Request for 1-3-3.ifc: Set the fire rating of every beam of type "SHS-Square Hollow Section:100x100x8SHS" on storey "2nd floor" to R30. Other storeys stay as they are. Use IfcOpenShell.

First a look at what the model holds.

```python
import ifcopenshell
import ifcopenshell.util.element

model = ifcopenshell.open("1-3-3.ifc")
print(model.schema)
storey = next(s for s in model.by_type("IfcBuildingStorey") if s.Name == "2nd floor")
beams = [e for e in ifcopenshell.util.element.get_decomposition(storey) if e.is_a("IfcBeam")]
seen = {}
for e in beams:
    element_type = ifcopenshell.util.element.get_type(e)
    key = (element_type.Name if element_type != e and element_type else None, ifcopenshell.util.element.get_pset(e, "Pset_BeamCommon", "FireRating"))
    seen[key] = seen.get(key, 0) + 1
for (name, value), count in sorted(seen.items(), key=str):
    print(count, "x", name, "|", value)
```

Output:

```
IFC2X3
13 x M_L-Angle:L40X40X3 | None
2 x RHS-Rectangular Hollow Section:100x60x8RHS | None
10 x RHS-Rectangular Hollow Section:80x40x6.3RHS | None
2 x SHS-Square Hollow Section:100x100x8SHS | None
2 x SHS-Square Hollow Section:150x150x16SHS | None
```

```python
import ifcopenshell
import ifcopenshell.api.pset
import ifcopenshell.util.element

model = ifcopenshell.open("1-3-3.ifc")

storey = next(s for s in model.by_type("IfcBuildingStorey") if s.Name == "2nd floor")
beams = [e for e in ifcopenshell.util.element.get_decomposition(storey) if e.is_a("IfcBeam")]

count = 0
for e in beams:
    element_type = ifcopenshell.util.element.get_type(e)
    if element_type in (None, e) or element_type.Name != "SHS-Square Hollow Section:100x100x8SHS":
        continue
    # add_pset returns the element's existing set when there is one.
    pset = ifcopenshell.api.pset.add_pset(model, product=e, name="Pset_BeamCommon")
    ifcopenshell.api.pset.edit_pset(model, pset=pset, properties={"FireRating": "R30"})
    count += 1

print(count, "beams updated")

model.write("1-3-3_edited.ifc")
```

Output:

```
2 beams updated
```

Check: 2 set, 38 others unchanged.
